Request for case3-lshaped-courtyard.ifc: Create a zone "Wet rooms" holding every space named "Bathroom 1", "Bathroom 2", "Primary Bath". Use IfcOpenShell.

First a look at what the model holds.

```python
import ifcopenshell

model = ifcopenshell.open("case3-lshaped-courtyard.ifc")
print(model.schema)
seen = {}
for space in model.by_type("IfcSpace"):
    seen[space.Name] = seen.get(space.Name, 0) + 1
for name, count in sorted(seen.items(), key=str):
    print(count, "x", name)
print("zones:", [z.Name for z in model.by_type("IfcZone")][:20])
```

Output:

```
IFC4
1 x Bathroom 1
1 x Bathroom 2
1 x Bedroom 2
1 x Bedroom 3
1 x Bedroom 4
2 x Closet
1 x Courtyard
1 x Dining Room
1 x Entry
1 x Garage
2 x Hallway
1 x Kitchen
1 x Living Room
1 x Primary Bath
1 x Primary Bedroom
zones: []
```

```python
import ifcopenshell
import ifcopenshell.api.group
import ifcopenshell.api.root

model = ifcopenshell.open("case3-lshaped-courtyard.ifc")

names = {"Bathroom 1", "Bathroom 2", "Primary Bath"}
spaces = [s for s in model.by_type("IfcSpace") if s.Name in names]

zone = ifcopenshell.api.root.create_entity(model, ifc_class="IfcZone", name="Wet rooms")
ifcopenshell.api.group.assign_group(model, products=spaces, group=zone)
print(len(spaces), "spaces in", zone.Name)

model.write("case3-lshaped-courtyard-out.ifc")
```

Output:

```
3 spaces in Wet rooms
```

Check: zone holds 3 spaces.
